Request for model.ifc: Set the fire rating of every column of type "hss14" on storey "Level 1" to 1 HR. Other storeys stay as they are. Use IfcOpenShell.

First a look at what the model holds.

```python
import ifcopenshell
import ifcopenshell.util.element

model = ifcopenshell.open("model.ifc")
print(model.schema)
storey = next(s for s in model.by_type("IfcBuildingStorey") if s.Name == "Level 1")
columns = [e for e in ifcopenshell.util.element.get_decomposition(storey) if e.is_a("IfcColumn")]
seen = {}
for e in columns:
    element_type = ifcopenshell.util.element.get_type(e)
    key = (element_type.Name if element_type != e and element_type else None, ifcopenshell.util.element.get_pset(e, "Pset_ColumnCommon", "FireRating"))
    seen[key] = seen.get(key, 0) + 1
for (name, value), count in sorted(seen.items(), key=str):
    print(count, "x", name, "|", value)
```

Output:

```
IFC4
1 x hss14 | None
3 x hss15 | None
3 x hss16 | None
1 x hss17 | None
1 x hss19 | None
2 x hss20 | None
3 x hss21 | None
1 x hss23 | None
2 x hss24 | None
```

```python
import ifcopenshell
import ifcopenshell.api.pset
import ifcopenshell.util.element

model = ifcopenshell.open("model.ifc")

storey = next(s for s in model.by_type("IfcBuildingStorey") if s.Name == "Level 1")
columns = [e for e in ifcopenshell.util.element.get_decomposition(storey) if e.is_a("IfcColumn")]

count = 0
for e in columns:
    element_type = ifcopenshell.util.element.get_type(e)
    if element_type in (None, e) or element_type.Name != "hss14":
        continue
    # add_pset returns the element's existing set when there is one.
    pset = ifcopenshell.api.pset.add_pset(model, product=e, name="Pset_ColumnCommon")
    ifcopenshell.api.pset.edit_pset(model, pset=pset, properties={"FireRating": "1 HR"})
    count += 1

print(count, "columns updated")

model.write("model_updated.ifc")
```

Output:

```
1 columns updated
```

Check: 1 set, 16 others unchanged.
